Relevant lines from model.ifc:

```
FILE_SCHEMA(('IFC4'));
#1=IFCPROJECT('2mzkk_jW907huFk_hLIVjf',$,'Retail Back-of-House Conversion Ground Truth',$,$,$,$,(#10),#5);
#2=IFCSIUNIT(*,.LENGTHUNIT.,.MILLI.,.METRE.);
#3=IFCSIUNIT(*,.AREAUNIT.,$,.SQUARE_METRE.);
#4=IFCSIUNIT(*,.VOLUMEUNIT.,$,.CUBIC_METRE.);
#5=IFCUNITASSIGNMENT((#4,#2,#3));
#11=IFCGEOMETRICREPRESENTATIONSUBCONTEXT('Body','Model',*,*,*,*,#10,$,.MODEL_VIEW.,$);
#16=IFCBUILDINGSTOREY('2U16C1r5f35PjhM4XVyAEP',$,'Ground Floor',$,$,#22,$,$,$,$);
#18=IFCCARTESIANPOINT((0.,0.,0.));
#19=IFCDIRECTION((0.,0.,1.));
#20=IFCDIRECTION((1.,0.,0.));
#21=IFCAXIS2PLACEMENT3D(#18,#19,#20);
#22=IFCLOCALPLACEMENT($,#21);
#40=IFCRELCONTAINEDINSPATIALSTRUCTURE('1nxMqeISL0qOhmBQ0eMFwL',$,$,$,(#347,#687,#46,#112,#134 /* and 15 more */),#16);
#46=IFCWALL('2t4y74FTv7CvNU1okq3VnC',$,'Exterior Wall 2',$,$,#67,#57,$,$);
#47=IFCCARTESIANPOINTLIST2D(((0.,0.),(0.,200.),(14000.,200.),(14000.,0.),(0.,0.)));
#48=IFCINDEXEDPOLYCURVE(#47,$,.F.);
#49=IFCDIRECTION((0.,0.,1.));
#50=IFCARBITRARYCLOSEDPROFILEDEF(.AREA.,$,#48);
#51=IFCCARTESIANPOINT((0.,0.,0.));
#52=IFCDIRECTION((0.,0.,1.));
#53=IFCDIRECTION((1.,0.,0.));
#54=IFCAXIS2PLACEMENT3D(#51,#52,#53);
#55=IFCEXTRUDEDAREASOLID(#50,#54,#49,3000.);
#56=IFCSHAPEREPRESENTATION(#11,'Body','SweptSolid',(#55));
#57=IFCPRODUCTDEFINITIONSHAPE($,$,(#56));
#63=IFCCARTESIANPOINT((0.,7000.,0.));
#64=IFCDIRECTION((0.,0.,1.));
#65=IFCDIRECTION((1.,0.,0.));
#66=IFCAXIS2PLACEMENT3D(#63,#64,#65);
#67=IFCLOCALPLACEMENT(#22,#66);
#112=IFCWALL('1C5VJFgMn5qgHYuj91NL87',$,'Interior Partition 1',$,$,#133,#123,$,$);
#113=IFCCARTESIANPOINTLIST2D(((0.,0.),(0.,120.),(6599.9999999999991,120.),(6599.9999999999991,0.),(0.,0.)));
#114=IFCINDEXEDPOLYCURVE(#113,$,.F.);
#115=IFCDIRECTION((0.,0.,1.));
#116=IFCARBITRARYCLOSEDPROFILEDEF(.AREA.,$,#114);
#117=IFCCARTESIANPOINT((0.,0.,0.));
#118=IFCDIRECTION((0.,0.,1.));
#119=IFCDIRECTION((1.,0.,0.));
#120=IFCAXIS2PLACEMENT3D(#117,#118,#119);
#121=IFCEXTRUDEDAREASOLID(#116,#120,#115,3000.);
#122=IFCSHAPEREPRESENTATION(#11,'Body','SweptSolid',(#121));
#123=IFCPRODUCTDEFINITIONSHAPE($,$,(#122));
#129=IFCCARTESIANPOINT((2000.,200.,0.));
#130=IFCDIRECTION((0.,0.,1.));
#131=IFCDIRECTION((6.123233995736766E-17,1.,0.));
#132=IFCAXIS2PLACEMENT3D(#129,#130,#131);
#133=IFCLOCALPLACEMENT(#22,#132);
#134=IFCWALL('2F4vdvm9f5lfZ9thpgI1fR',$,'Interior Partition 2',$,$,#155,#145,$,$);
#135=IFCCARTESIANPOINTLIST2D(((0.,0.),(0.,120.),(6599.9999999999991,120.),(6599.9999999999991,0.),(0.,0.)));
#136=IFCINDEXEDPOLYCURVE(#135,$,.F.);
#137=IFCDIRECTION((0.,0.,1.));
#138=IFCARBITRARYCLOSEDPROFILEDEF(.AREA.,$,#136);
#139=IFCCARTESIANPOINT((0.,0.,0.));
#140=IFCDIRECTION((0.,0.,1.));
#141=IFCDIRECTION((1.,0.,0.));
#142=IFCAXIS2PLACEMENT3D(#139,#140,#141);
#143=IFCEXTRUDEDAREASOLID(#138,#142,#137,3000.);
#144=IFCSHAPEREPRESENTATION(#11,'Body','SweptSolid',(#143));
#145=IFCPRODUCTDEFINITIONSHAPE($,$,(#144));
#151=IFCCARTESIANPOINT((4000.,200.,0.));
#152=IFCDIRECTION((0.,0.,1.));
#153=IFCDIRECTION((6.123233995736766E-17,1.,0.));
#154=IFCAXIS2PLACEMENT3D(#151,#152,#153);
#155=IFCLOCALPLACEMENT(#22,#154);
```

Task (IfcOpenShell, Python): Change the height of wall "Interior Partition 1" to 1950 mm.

```python
import ifcopenshell
import ifcopenshell.geom
import ifcopenshell.util.representation
import ifcopenshell.util.shape

model = ifcopenshell.open("model.ifc")
settings = ifcopenshell.geom.settings()


def volume(element):
    """Net volume in cubic metres, openings subtracted."""
    shape = ifcopenshell.geom.create_shape(settings, element)
    return ifcopenshell.util.shape.get_volume(shape.geometry)


wall = model.by_guid("1C5VJFgMn5qgHYuj91NL87")
before = volume(wall)

body = ifcopenshell.util.representation.get_representation(wall, "Model", "Body")
solid = body.Items[0]
old_height = solid.Depth
solid.Depth = 1950.0
after = volume(wall)

print(f"height {old_height:g} -> {solid.Depth:g}, volume {before:.3f} -> {after:.3f} m3")

model.write("model_updated.ifc")
```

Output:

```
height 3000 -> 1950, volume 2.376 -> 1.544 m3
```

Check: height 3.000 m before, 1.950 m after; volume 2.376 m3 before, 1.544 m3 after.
